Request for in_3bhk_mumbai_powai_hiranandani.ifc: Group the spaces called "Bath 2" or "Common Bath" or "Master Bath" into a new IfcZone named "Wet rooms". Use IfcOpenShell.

First a look at what the model holds.

```python
import ifcopenshell

model = ifcopenshell.open("in_3bhk_mumbai_powai_hiranandani.ifc")
print(model.schema)
seen = {}
for space in model.by_type("IfcSpace"):
    seen[space.LongName] = seen.get(space.LongName, 0) + 1
for name, count in sorted(seen.items(), key=str):
    print(count, "x", name)
print("zones:", [z.Name for z in model.by_type("IfcZone")][:20])
```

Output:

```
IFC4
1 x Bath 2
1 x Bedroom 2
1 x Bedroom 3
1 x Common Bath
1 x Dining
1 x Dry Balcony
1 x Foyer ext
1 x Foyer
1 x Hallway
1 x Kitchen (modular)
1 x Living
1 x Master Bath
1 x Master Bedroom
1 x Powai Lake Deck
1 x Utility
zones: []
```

```python
import ifcopenshell
import ifcopenshell.api.group
import ifcopenshell.api.root

model = ifcopenshell.open("in_3bhk_mumbai_powai_hiranandani.ifc")

names = {"Bath 2", "Common Bath", "Master Bath"}
spaces = [s for s in model.by_type("IfcSpace") if s.LongName in names]

zone = ifcopenshell.api.root.create_entity(model, ifc_class="IfcZone", name="Wet rooms")
ifcopenshell.api.group.assign_group(model, products=spaces, group=zone)
print(len(spaces), "spaces in", zone.Name)

model.write("in_3bhk_mumbai_powai_hiranandani-out.ifc")
```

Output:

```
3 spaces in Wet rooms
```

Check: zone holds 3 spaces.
